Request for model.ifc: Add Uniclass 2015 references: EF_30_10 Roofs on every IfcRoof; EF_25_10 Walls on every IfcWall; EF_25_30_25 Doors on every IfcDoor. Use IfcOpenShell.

First a look at what the model holds.

```python
import ifcopenshell

model = ifcopenshell.open("model.ifc")
print(model.schema)
print("classifications:", [c.Name for c in model.by_type("IfcClassification")])
for ifc_class in ("IfcDoor", "IfcRoof", "IfcStair", "IfcWall", "IfcWindow"):
    print(ifc_class, len(model.by_type(ifc_class)))
```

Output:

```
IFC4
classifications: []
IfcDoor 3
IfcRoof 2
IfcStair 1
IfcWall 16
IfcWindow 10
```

```python
import ifcopenshell
import ifcopenshell.api.classification

model = ifcopenshell.open("model.ifc")

system = ifcopenshell.api.classification.add_classification(model, classification="Uniclass 2015")

codes = {
    "IfcRoof": ("EF_30_10", "Roofs"),
    "IfcWall": ("EF_25_10", "Walls"),
    "IfcDoor": ("EF_25_30_25", "Doors"),
}
for ifc_class, (code, name) in codes.items():
    products = model.by_type(ifc_class)
    ifcopenshell.api.classification.add_reference(
        model, products=products, classification=system, identification=code, name=name
    )
    print(code, len(products))

model.write("model_updated.ifc")
```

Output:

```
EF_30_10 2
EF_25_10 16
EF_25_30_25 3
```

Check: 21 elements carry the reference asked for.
